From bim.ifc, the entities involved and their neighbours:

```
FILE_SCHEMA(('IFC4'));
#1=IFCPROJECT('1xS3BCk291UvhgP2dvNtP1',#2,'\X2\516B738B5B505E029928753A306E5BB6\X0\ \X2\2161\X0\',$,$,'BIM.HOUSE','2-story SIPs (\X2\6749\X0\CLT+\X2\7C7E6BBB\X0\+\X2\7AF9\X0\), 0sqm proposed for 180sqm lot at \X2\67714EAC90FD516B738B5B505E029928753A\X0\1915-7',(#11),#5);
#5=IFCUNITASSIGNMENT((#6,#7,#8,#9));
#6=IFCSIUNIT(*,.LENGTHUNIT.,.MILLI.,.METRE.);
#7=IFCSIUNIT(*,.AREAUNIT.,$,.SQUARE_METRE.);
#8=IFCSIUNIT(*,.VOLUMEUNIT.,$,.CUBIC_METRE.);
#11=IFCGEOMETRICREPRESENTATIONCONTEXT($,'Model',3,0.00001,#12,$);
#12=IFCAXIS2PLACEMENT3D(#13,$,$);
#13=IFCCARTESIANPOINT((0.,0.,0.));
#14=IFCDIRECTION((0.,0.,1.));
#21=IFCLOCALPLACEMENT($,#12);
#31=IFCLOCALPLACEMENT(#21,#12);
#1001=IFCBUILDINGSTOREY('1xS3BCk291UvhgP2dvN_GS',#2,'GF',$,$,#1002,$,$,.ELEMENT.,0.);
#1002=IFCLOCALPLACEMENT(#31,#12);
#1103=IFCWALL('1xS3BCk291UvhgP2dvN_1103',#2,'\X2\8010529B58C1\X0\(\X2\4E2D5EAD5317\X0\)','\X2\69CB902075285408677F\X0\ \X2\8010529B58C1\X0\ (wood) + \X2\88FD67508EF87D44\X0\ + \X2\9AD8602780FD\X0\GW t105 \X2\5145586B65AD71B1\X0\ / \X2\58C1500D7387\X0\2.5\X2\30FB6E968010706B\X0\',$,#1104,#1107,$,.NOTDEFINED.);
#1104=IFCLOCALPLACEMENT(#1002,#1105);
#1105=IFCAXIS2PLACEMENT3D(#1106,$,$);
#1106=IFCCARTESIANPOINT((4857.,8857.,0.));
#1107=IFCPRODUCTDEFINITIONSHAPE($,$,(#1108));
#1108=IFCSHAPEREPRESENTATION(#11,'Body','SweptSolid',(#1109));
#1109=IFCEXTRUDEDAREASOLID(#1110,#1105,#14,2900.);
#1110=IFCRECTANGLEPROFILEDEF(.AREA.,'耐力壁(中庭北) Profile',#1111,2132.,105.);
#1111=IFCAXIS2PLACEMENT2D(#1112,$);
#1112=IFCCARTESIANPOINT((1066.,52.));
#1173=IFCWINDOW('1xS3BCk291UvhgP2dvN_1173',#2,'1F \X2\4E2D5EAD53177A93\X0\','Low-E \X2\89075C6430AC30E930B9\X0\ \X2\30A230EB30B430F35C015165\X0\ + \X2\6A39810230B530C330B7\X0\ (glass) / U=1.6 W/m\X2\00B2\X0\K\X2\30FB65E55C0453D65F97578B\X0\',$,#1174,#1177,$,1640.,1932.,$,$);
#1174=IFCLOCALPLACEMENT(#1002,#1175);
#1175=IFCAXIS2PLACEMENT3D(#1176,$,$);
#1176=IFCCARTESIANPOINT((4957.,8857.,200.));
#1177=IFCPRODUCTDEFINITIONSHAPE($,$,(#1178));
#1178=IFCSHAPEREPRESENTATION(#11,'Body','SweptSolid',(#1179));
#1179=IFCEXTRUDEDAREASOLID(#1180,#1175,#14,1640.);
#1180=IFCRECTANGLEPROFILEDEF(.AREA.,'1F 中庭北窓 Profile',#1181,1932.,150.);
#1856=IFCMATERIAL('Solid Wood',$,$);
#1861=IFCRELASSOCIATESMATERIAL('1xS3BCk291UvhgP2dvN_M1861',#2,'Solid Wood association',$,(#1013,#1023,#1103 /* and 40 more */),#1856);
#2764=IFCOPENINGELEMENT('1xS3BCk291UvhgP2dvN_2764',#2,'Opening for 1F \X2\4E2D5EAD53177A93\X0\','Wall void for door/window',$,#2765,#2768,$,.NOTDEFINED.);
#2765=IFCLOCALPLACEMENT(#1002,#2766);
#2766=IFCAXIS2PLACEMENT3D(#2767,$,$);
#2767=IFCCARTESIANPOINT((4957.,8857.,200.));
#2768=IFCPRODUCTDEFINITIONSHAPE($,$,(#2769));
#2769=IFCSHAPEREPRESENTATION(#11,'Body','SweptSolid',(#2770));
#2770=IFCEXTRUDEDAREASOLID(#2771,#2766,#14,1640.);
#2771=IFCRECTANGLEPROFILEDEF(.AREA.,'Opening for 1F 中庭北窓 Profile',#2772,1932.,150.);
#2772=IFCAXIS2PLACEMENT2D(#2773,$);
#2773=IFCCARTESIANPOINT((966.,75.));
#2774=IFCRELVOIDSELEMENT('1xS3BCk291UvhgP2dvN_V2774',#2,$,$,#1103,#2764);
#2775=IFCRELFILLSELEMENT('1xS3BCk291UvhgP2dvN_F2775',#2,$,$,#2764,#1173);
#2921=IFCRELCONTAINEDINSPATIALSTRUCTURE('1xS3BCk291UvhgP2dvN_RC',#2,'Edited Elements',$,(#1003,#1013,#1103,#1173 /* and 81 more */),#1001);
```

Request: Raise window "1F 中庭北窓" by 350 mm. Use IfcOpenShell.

```python
import numpy as np
import ifcopenshell
import ifcopenshell.api.geometry
import ifcopenshell.util.placement
import ifcopenshell.util.unit

model = ifcopenshell.open("bim.ifc")
unit_scale = ifcopenshell.util.unit.calculate_unit_scale(model)

window = model.by_guid("1xS3BCk291UvhgP2dvN_1173")
opening = window.FillsVoids[0].RelatingOpeningElement
dz = 0.35 / unit_scale

shift = np.array([0.0, 0.0, dz])
# The window is not placed relative to its opening, so move both.
for product in (opening, window):
    matrix = ifcopenshell.util.placement.get_local_placement(product.ObjectPlacement)
    matrix[:3, 3] += shift
    ifcopenshell.api.geometry.edit_object_placement(model, product=product, matrix=matrix, is_si=False)

print(f"moved by {dz * unit_scale:+.3f} m")

model.write("bim-out.ifc")
```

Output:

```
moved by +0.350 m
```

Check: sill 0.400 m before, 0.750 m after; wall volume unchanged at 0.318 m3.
